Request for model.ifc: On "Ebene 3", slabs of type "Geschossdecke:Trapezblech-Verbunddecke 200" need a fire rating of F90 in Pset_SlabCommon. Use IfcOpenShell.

First a look at what the model holds.

```python
import ifcopenshell
import ifcopenshell.util.element

model = ifcopenshell.open("model.ifc")
print(model.schema)
storey = next(s for s in model.by_type("IfcBuildingStorey") if s.Name == "Ebene 3")
slabs = [e for e in ifcopenshell.util.element.get_decomposition(storey) if e.is_a("IfcSlab")]
seen = {}
for e in slabs:
    element_type = ifcopenshell.util.element.get_type(e)
    key = (element_type.Name if element_type != e and element_type else None, ifcopenshell.util.element.get_pset(e, "Pset_SlabCommon", "FireRating"))
    seen[key] = seen.get(key, 0) + 1
for (name, value), count in sorted(seen.items(), key=str):
    print(count, "x", name, "|", value)
```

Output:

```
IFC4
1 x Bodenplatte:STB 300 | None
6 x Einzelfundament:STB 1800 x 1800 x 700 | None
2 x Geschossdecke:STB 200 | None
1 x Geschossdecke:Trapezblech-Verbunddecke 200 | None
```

```python
import ifcopenshell
import ifcopenshell.api.pset
import ifcopenshell.util.element

model = ifcopenshell.open("model.ifc")

storey = next(s for s in model.by_type("IfcBuildingStorey") if s.Name == "Ebene 3")
slabs = [e for e in ifcopenshell.util.element.get_decomposition(storey) if e.is_a("IfcSlab")]

count = 0
for e in slabs:
    element_type = ifcopenshell.util.element.get_type(e)
    if element_type in (None, e) or element_type.Name != "Geschossdecke:Trapezblech-Verbunddecke 200":
        continue
    # add_pset returns the element's existing set when there is one.
    pset = ifcopenshell.api.pset.add_pset(model, product=e, name="Pset_SlabCommon")
    ifcopenshell.api.pset.edit_pset(model, pset=pset, properties={"FireRating": "F90"})
    count += 1

print(count, "slabs updated")

model.write("model_updated.ifc")
```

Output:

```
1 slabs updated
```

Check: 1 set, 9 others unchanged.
